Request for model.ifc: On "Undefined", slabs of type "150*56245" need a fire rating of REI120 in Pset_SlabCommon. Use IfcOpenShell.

First a look at what the model holds.

```python
import ifcopenshell
import ifcopenshell.util.element

model = ifcopenshell.open("model.ifc")
print(model.schema)
storey = next(s for s in model.by_type("IfcBuildingStorey") if s.Name == "Undefined")
slabs = [e for e in ifcopenshell.util.element.get_decomposition(storey) if e.is_a("IfcSlab")]
seen = {}
for e in slabs:
    element_type = ifcopenshell.util.element.get_type(e)
    key = (element_type.Name if element_type != e and element_type else None, ifcopenshell.util.element.get_pset(e, "Pset_SlabCommon", "FireRating"))
    seen[key] = seen.get(key, 0) + 1
for (name, value), count in sorted(seen.items(), key=str):
    print(count, "x", name, "|", value)
```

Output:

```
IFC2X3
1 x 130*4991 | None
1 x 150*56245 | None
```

```python
import ifcopenshell
import ifcopenshell.api.pset
import ifcopenshell.util.element

model = ifcopenshell.open("model.ifc")

storey = next(s for s in model.by_type("IfcBuildingStorey") if s.Name == "Undefined")
slabs = [e for e in ifcopenshell.util.element.get_decomposition(storey) if e.is_a("IfcSlab")]

count = 0
for e in slabs:
    element_type = ifcopenshell.util.element.get_type(e)
    if element_type in (None, e) or element_type.Name != "150*56245":
        continue
    found = ifcopenshell.util.element.get_pset(e, "Pset_SlabCommon", should_inherit=False)
    if found:
        pset = model.by_id(found["id"])
        if len(ifcopenshell.util.element.get_elements_by_pset(pset)) > 1:
            pset = ifcopenshell.api.pset.unshare_pset(model, products=[e], pset=pset)[0]
    else:
        pset = ifcopenshell.api.pset.add_pset(model, product=e, name="Pset_SlabCommon")
    ifcopenshell.api.pset.edit_pset(model, pset=pset, properties={"FireRating": "REI120"})
    count += 1

print(count, "slabs updated")

model.write("model-out.ifc")
```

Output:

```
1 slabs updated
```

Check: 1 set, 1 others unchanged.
